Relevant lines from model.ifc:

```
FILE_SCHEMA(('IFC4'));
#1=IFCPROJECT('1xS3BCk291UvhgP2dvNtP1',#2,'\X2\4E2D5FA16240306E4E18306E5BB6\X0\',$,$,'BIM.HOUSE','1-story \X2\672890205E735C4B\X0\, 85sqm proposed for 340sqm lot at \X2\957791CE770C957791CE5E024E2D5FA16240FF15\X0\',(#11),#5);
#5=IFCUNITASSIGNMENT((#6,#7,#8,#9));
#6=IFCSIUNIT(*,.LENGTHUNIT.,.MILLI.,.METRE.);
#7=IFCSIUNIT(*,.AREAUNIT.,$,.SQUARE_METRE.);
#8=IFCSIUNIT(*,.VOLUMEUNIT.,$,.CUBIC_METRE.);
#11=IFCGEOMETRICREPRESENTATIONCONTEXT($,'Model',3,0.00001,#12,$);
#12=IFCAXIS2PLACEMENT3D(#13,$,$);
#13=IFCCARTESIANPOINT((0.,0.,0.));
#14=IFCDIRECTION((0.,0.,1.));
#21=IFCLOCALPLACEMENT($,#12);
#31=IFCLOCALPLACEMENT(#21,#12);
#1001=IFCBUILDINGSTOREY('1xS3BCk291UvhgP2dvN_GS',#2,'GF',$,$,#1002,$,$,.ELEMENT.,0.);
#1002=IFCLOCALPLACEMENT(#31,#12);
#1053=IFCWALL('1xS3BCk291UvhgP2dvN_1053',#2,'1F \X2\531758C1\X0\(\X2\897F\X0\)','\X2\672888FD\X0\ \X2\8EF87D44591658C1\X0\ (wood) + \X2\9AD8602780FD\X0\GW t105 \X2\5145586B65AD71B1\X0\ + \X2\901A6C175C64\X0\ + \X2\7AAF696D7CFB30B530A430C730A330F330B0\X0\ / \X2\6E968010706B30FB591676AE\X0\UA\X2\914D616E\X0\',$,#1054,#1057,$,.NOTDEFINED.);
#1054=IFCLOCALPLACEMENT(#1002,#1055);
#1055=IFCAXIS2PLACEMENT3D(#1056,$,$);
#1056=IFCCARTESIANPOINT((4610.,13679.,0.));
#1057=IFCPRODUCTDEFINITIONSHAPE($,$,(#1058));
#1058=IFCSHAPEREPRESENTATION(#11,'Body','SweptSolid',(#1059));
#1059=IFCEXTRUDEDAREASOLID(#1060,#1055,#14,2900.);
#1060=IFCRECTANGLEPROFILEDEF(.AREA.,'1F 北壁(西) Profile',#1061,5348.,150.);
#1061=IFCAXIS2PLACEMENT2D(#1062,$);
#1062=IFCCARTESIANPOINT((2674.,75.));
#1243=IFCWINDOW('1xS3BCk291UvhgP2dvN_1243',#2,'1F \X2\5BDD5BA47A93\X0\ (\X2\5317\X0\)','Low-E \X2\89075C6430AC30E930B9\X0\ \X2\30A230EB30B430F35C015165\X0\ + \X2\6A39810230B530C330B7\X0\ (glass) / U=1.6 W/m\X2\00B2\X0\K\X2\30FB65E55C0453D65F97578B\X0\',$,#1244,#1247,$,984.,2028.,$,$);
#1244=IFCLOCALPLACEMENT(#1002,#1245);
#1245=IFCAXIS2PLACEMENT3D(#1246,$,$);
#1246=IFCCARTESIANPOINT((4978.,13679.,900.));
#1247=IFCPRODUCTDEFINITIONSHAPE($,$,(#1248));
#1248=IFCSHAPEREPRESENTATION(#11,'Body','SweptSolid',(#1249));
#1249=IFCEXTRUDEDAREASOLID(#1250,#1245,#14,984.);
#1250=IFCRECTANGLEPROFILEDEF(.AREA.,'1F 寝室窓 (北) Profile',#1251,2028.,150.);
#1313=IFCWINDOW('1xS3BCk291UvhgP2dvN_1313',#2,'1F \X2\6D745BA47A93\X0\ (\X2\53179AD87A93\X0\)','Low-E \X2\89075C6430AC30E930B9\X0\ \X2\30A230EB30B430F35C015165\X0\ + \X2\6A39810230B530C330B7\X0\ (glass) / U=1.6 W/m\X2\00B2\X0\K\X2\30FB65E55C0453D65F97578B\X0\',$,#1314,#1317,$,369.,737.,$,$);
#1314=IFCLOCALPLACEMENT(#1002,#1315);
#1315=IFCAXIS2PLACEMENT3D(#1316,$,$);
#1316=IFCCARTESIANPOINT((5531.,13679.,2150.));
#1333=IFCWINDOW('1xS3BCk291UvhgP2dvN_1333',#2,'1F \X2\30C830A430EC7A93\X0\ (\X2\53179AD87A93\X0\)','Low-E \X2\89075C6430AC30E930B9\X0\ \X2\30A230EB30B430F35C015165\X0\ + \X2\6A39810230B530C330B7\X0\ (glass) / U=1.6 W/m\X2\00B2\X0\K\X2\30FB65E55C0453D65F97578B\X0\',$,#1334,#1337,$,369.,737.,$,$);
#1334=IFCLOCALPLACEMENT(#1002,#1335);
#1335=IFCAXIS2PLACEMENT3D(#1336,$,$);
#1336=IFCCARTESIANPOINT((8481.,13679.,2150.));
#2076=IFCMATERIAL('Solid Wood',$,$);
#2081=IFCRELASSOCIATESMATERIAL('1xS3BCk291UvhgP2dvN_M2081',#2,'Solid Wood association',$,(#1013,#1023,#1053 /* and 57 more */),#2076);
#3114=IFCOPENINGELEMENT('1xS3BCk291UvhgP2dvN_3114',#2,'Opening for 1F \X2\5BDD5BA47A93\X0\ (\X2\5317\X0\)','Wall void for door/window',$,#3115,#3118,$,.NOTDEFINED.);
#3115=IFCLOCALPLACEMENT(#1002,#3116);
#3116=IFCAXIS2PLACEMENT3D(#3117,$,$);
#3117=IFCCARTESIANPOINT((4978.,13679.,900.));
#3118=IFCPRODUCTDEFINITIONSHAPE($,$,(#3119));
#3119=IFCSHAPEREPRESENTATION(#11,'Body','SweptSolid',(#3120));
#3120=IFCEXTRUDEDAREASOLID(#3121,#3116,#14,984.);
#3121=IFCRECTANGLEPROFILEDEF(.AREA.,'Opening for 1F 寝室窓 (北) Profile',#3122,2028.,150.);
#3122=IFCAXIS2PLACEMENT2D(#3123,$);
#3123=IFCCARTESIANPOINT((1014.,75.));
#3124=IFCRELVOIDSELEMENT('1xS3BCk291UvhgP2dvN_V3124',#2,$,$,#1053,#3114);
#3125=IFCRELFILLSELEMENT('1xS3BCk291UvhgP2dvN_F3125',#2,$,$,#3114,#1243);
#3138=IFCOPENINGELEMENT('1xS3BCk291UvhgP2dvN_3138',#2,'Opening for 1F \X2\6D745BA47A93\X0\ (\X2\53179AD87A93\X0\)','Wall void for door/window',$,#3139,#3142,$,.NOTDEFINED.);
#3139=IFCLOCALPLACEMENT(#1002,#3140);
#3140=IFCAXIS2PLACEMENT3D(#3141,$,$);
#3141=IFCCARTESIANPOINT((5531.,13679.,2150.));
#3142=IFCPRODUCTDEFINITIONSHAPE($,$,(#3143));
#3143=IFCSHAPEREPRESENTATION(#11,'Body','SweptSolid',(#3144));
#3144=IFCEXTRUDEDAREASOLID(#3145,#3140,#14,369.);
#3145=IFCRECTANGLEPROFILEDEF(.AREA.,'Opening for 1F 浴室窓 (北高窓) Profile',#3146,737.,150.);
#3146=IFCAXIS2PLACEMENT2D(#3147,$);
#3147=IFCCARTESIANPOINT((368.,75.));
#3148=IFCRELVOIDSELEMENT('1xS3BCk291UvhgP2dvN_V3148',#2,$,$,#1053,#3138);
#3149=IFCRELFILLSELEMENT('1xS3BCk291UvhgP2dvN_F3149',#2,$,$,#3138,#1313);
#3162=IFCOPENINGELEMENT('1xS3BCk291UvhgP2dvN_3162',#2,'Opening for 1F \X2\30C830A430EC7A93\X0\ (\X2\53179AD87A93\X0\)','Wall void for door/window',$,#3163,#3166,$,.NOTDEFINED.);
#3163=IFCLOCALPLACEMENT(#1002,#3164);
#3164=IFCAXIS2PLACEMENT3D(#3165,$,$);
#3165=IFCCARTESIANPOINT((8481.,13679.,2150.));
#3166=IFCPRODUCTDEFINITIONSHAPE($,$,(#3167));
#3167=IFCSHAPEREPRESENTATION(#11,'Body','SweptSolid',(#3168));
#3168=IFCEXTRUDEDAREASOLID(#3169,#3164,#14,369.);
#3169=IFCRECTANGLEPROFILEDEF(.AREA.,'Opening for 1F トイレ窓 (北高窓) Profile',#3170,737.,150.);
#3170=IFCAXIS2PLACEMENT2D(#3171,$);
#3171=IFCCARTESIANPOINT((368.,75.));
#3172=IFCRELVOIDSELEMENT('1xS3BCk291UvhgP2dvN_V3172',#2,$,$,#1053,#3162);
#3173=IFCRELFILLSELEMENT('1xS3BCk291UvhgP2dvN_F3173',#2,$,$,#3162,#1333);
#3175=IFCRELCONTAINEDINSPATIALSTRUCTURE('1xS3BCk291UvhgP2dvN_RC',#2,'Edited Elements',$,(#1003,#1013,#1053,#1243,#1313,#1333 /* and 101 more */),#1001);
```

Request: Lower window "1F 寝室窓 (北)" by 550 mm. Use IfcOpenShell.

```python
import numpy as np
import ifcopenshell
import ifcopenshell.api.geometry
import ifcopenshell.util.placement
import ifcopenshell.util.unit

model = ifcopenshell.open("model.ifc")
unit_scale = ifcopenshell.util.unit.calculate_unit_scale(model)

window = model.by_guid("1xS3BCk291UvhgP2dvN_1243")
opening = window.FillsVoids[0].RelatingOpeningElement
dz = -0.55 / unit_scale

shift = np.array([0.0, 0.0, dz])
# The window is not placed relative to its opening, so move both.
for product in (opening, window):
    matrix = ifcopenshell.util.placement.get_local_placement(product.ObjectPlacement)
    matrix[:3, 3] += shift
    ifcopenshell.api.geometry.edit_object_placement(model, product=product, matrix=matrix, is_si=False)

print(f"moved by {dz * unit_scale:+.3f} m")

model.write("model_v2.ifc")
```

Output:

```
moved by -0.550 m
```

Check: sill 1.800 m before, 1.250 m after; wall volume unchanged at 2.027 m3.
